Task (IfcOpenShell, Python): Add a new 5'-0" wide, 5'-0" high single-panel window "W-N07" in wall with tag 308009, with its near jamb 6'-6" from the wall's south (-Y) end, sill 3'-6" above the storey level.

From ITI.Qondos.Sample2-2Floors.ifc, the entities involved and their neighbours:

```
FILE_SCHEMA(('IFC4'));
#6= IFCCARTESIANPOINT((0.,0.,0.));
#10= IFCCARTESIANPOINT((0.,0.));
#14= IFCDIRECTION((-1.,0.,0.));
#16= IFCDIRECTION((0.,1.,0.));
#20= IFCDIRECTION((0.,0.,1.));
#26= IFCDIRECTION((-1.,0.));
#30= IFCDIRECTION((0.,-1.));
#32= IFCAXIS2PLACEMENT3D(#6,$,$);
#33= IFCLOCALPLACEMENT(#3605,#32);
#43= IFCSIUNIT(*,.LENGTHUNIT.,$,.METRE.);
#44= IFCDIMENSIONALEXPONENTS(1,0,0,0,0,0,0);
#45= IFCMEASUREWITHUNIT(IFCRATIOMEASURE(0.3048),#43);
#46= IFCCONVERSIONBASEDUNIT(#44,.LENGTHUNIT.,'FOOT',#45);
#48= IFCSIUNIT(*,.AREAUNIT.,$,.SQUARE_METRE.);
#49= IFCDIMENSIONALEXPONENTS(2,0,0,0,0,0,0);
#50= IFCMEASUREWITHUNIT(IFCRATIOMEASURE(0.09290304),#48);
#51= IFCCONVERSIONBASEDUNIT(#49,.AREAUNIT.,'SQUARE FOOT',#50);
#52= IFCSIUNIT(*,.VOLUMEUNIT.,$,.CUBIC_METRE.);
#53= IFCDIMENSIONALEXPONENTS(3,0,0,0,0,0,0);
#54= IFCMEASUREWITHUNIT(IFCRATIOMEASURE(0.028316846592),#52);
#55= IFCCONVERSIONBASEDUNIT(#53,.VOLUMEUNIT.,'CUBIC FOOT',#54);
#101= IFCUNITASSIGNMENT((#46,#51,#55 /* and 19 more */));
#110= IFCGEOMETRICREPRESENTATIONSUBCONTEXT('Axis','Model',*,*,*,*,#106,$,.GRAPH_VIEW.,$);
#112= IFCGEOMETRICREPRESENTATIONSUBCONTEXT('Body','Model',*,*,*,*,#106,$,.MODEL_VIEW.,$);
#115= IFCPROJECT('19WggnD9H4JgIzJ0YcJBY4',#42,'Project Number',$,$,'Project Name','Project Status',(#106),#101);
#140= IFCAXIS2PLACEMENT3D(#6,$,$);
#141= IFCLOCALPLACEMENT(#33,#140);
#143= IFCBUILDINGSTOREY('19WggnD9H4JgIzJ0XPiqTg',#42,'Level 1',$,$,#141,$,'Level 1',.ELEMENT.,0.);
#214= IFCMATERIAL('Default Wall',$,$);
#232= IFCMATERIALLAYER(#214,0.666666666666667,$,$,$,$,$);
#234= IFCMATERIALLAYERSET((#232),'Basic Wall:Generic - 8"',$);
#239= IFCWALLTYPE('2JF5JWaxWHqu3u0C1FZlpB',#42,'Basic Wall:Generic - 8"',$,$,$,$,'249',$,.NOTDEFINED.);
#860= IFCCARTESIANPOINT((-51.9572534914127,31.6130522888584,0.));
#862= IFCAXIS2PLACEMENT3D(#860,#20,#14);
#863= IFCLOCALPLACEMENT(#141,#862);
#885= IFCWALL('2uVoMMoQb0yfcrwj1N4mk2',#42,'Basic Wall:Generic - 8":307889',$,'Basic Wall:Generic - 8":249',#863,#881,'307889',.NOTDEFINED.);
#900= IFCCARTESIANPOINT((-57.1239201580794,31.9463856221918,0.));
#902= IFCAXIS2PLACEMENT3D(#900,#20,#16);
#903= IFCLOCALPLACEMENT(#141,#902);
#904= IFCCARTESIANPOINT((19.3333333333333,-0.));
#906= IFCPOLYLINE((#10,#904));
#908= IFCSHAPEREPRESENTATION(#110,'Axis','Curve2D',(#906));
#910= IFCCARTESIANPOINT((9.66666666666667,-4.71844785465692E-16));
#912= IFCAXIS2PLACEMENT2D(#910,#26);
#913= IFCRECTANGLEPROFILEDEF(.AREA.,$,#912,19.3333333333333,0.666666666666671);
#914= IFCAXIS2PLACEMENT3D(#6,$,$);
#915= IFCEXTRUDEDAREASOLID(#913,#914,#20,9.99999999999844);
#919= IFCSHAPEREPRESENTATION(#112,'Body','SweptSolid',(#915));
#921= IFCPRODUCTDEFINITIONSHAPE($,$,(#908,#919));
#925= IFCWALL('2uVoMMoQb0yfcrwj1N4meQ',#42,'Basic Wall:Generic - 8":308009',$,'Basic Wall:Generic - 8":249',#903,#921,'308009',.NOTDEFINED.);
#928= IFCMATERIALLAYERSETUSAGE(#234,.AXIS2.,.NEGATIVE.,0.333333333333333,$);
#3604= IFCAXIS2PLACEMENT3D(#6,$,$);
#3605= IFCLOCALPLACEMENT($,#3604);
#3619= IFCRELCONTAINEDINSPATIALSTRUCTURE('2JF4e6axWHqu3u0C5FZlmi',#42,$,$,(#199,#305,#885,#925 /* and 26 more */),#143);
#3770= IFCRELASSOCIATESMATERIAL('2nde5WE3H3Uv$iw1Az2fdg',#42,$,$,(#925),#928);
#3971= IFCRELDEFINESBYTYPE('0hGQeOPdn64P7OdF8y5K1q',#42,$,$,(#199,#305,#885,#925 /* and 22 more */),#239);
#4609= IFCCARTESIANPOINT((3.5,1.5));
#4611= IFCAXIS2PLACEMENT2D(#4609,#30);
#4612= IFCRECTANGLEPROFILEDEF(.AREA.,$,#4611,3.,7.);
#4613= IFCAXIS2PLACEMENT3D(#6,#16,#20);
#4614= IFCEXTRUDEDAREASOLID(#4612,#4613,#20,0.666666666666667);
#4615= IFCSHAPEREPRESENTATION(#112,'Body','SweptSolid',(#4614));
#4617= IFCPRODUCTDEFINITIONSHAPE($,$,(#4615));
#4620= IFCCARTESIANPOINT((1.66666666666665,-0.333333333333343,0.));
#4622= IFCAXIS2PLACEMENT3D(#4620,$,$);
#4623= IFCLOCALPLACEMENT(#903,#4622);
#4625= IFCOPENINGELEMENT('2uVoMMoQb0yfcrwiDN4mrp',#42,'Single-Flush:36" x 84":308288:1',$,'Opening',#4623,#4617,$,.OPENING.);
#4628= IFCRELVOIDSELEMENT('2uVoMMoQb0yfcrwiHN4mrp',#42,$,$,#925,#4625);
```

```python
import numpy as np
import ifcopenshell
import ifcopenshell.api.feature
import ifcopenshell.api.geometry
import ifcopenshell.api.root
import ifcopenshell.api.spatial
import ifcopenshell.geom
import ifcopenshell.util.element
import ifcopenshell.util.placement
import ifcopenshell.util.representation
import ifcopenshell.util.shape
import ifcopenshell.util.unit

model = ifcopenshell.open("ITI.Qondos.Sample2-2Floors.ifc")
unit_scale = ifcopenshell.util.unit.calculate_unit_scale(model)
settings = ifcopenshell.geom.settings()


def volume(element):
    """Net volume in cubic metres, openings subtracted."""
    shape = ifcopenshell.geom.create_shape(settings, element)
    return ifcopenshell.util.shape.get_volume(shape.geometry)


wall = model.by_guid("2uVoMMoQb0yfcrwj1N4meQ")
storey = ifcopenshell.util.element.get_container(wall, ifc_class="IfcBuildingStorey")
context = ifcopenshell.util.representation.get_context(model, "Model", "Body", "MODEL_VIEW")
before = volume(wall)

width, height, from_end, sill = 1.524, 1.524, 1.9812, 1.0668  # metres

# The wall runs along its own X axis, and the end named is its -X end.
wall_shape = ifcopenshell.geom.create_shape(settings, wall)
x, y, z = ifcopenshell.util.shape.get_vertices(wall_shape.geometry).T
start = x.min() + from_end
face, thickness = float(y.min()), float(y.max() - y.min())
wall_matrix = ifcopenshell.util.placement.get_local_placement(wall.ObjectPlacement)
level = ifcopenshell.util.placement.get_local_placement(storey.ObjectPlacement)[2, 3]


def in_wall(x, y):
    """Placement at x, y metres in the wall's axes, at sill height."""
    matrix = wall_matrix.copy()
    matrix[:, 3] = wall_matrix @ np.array([x / unit_scale, y / unit_scale, 0.0, 1.0])
    matrix[2, 3] = level + sill / unit_scale
    return matrix


# Opening: a box that overshoots both wall faces by 50 mm.
opening = ifcopenshell.api.root.create_entity(model, ifc_class="IfcOpeningElement", predefined_type="OPENING")
box = ifcopenshell.api.geometry.add_wall_representation(
    model, context=context, length=width, height=height, thickness=thickness + 0.1
)
ifcopenshell.api.geometry.assign_representation(model, product=opening, representation=box)
ifcopenshell.api.geometry.edit_object_placement(model, product=opening, matrix=in_wall(start, face - 0.05), is_si=False)
ifcopenshell.api.feature.add_feature(model, feature=opening, element=wall)

window = ifcopenshell.api.root.create_entity(model, ifc_class="IfcWindow", name="W-N07", predefined_type="WINDOW")
window.OverallWidth, window.OverallHeight = width / unit_scale, height / unit_scale
window.PartitioningType = "SINGLE_PANEL"
body = ifcopenshell.api.geometry.add_window_representation(
    model,
    context=context,
    overall_width=window.OverallWidth,
    overall_height=window.OverallHeight,
    partition_type="SINGLE_PANEL",
)
ifcopenshell.api.geometry.assign_representation(model, product=window, representation=body)
ifcopenshell.api.spatial.assign_container(model, products=[window], relating_structure=storey)
ifcopenshell.api.feature.add_filling(model, opening=opening, element=window)

# Centre the window in the wall's thickness.
ifcopenshell.api.geometry.edit_object_placement(model, product=window, matrix=in_wall(start, face), is_si=False)
window_shape = ifcopenshell.geom.create_shape(settings, window)
depth = ifcopenshell.util.shape.get_vertices(window_shape.geometry)[:, 1]
offset = face + thickness / 2 - (depth.min() + depth.max()) / 2
ifcopenshell.api.geometry.edit_object_placement(model, product=window, matrix=in_wall(start, offset), is_si=False)

after = volume(wall)

print(f"wall volume {before:.3f} -> {after:.3f} m3")

model.write("ITI.Qondos.Sample2-2Floors_rev.ifc")
```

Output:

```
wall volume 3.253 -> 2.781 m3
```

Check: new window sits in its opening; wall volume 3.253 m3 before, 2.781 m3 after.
